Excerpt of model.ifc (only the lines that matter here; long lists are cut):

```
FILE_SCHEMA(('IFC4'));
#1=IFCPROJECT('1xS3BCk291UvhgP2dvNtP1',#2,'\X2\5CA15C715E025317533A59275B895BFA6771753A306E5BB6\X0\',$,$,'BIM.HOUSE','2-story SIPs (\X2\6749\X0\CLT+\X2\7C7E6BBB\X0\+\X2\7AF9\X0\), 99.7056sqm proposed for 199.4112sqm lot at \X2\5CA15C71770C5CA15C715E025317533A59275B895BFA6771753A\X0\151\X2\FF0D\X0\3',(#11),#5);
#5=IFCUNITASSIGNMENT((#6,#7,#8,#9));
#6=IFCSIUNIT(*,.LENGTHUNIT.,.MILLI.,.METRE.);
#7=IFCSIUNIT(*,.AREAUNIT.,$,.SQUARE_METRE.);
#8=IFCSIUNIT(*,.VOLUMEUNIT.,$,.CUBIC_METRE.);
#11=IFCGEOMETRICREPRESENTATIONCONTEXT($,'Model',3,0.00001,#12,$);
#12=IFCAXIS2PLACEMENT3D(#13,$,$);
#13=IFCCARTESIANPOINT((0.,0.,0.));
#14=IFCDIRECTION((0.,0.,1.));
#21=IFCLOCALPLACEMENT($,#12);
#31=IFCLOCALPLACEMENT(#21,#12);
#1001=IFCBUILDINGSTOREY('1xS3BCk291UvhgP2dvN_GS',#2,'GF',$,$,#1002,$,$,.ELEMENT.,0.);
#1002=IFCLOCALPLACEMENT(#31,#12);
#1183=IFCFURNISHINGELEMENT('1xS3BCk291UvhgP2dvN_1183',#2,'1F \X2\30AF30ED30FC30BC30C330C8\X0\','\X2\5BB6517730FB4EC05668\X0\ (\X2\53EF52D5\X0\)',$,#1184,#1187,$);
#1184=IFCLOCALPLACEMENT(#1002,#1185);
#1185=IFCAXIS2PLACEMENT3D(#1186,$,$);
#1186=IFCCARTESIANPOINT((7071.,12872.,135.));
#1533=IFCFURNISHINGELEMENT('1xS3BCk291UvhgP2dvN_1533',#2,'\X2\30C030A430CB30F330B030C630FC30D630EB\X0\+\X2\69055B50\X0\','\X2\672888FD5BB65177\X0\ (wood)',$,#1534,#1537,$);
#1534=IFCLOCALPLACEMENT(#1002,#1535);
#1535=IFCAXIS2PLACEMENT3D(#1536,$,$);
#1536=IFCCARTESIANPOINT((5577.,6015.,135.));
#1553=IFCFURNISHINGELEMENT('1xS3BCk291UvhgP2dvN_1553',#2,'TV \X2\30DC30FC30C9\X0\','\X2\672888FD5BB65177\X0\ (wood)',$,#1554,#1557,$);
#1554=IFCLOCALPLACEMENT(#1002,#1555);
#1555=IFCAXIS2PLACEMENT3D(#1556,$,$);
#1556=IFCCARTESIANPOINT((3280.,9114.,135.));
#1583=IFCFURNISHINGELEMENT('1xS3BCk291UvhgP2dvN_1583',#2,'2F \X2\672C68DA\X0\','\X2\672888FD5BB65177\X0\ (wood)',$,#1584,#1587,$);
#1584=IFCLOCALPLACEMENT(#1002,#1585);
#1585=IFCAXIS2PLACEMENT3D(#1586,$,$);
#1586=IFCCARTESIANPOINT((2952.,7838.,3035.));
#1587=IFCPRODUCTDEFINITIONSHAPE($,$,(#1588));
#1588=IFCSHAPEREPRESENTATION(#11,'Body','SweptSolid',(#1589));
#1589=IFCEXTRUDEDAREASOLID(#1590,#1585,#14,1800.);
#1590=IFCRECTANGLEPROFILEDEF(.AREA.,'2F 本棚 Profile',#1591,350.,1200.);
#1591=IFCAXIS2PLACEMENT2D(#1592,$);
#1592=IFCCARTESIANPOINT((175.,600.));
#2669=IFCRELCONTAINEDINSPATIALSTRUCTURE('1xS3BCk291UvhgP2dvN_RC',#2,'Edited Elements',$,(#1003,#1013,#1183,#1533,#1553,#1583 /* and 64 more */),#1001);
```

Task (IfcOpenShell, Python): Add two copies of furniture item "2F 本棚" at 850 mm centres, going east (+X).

```python
import numpy as np
import ifcopenshell
import ifcopenshell.api.geometry
import ifcopenshell.api.root
import ifcopenshell.util.element
import ifcopenshell.util.placement

model = ifcopenshell.open("model.ifc")


def reuse_history(source, copy):
    """copy_class also copies each property set's owner history, people and application; keep the originals."""
    for rel in copy.IsDefinedBy:
        if rel.is_a("IfcRelDefinesByProperties") and (history := rel.RelatingPropertyDefinition.OwnerHistory):
            rel.RelatingPropertyDefinition.OwnerHistory = source.OwnerHistory
            ifcopenshell.util.element.remove_deep2(model, history)


source = model.by_guid("1xS3BCk291UvhgP2dvN_1583")
base = ifcopenshell.util.placement.get_local_placement(source.ObjectPlacement)
step = np.array([1.0, 0.0, 0.0]) * 850.0

for i in range(1, 3):
    copy = ifcopenshell.api.root.copy_class(model, product=source)
    copy.Representation = ifcopenshell.util.element.copy_deep(
        model, source.Representation, exclude=["IfcGeometricRepresentationContext", "IfcRepresentationMap"]
    )
    reuse_history(source, copy)
    matrix = base.copy()
    matrix[:3, 3] += i * step
    print("added at", matrix[:3, 3].round(3) + 0.0)
    ifcopenshell.api.geometry.edit_object_placement(model, product=copy, matrix=matrix, is_si=False)

model.write("model_edited.ifc")
```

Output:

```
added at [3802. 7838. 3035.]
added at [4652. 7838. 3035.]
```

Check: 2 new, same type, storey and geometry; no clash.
